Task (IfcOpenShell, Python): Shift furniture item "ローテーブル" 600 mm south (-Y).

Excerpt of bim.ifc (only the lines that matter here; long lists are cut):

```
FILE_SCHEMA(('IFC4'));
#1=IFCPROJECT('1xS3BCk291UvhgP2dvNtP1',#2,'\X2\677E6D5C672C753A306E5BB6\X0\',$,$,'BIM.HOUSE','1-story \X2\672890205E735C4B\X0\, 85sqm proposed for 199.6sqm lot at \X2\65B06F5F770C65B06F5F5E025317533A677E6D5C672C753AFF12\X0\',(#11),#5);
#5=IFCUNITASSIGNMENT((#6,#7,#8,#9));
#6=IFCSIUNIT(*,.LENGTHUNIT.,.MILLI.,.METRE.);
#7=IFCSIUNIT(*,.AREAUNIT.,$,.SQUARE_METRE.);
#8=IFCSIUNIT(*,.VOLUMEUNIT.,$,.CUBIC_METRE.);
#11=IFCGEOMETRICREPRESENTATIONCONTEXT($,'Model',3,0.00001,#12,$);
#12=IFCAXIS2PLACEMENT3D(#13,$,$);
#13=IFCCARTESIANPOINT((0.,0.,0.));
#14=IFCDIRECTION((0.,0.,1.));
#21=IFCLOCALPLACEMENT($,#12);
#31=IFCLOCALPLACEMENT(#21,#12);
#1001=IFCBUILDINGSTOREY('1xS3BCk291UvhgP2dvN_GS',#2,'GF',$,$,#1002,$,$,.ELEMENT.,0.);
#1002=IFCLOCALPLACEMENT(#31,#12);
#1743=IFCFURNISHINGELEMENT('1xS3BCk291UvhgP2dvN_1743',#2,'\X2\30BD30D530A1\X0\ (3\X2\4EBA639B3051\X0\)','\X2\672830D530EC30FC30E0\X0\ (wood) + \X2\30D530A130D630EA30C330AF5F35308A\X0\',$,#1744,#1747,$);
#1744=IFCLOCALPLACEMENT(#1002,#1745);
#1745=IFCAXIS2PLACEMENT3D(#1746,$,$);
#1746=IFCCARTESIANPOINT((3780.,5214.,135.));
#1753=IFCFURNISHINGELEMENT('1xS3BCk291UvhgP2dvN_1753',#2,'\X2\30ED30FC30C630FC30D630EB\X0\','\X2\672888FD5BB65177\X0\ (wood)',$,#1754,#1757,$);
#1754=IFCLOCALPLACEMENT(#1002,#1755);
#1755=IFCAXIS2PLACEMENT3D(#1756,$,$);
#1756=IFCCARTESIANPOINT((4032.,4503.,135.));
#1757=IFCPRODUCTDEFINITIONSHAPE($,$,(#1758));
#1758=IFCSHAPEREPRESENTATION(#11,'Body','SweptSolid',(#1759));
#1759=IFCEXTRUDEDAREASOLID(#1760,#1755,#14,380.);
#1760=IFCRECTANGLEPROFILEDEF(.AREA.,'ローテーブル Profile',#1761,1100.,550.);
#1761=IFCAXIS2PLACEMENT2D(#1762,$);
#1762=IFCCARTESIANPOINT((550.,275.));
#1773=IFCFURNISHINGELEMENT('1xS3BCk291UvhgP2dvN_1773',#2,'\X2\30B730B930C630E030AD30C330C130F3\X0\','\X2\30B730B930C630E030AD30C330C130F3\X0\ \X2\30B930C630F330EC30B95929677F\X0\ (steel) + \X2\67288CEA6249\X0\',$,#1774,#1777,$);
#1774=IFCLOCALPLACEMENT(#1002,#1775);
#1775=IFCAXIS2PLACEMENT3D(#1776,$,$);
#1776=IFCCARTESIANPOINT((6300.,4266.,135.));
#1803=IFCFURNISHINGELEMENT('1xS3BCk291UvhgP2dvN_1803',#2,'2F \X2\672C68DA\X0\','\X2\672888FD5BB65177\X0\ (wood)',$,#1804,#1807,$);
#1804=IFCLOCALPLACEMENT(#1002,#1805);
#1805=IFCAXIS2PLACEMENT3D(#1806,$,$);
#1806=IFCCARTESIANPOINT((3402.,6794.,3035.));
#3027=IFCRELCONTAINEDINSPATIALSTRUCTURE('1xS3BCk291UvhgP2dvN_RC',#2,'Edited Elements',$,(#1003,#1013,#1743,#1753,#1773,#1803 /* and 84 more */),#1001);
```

```python
import ifcopenshell
import ifcopenshell.api.geometry
import ifcopenshell.util.placement
import ifcopenshell.util.unit

model = ifcopenshell.open("bim.ifc")
unit_scale = ifcopenshell.util.unit.calculate_unit_scale(model)

item = model.by_guid("1xS3BCk291UvhgP2dvN_1753")
matrix = ifcopenshell.util.placement.get_local_placement(item.ObjectPlacement)
matrix[1, 3] -= 0.6 / unit_scale
ifcopenshell.api.geometry.edit_object_placement(model, product=item, matrix=matrix, is_si=False)

print(ifcopenshell.util.placement.get_local_placement(item.ObjectPlacement).round(3) + 0.0)

model.write("bim-out.ifc")
```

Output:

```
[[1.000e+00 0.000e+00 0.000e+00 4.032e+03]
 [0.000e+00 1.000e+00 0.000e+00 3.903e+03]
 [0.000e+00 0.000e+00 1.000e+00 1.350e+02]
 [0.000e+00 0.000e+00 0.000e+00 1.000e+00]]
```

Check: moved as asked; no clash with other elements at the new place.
